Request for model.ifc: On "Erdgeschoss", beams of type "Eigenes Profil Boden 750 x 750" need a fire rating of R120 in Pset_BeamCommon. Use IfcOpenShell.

First a look at what the model holds.

```python
import ifcopenshell
import ifcopenshell.util.element

model = ifcopenshell.open("model.ifc")
print(model.schema)
storey = next(s for s in model.by_type("IfcBuildingStorey") if s.Name == "Erdgeschoss")
beams = [e for e in ifcopenshell.util.element.get_decomposition(storey) if e.is_a("IfcBeam")]
seen = {}
for e in beams:
    element_type = ifcopenshell.util.element.get_type(e)
    key = (element_type.Name if element_type != e and element_type else None, ifcopenshell.util.element.get_pset(e, "Pset_BeamCommon", "FireRating"))
    seen[key] = seen.get(key, 0) + 1
for (name, value), count in sorted(seen.items(), key=str):
    print(count, "x", name, "|", value)
```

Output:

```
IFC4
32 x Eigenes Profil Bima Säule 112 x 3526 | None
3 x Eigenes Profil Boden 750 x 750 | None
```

```python
import ifcopenshell
import ifcopenshell.api.pset
import ifcopenshell.util.element

model = ifcopenshell.open("model.ifc")

storey = next(s for s in model.by_type("IfcBuildingStorey") if s.Name == "Erdgeschoss")
beams = [e for e in ifcopenshell.util.element.get_decomposition(storey) if e.is_a("IfcBeam")]

count = 0
for e in beams:
    element_type = ifcopenshell.util.element.get_type(e)
    if element_type in (None, e) or element_type.Name != "Eigenes Profil Boden 750 x 750":
        continue
    # add_pset returns the element's existing set when there is one.
    pset = ifcopenshell.api.pset.add_pset(model, product=e, name="Pset_BeamCommon")
    ifcopenshell.api.pset.edit_pset(model, pset=pset, properties={"FireRating": "R120"})
    count += 1

print(count, "beams updated")

model.write("model_rev.ifc")
```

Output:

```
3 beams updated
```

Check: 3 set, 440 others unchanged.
